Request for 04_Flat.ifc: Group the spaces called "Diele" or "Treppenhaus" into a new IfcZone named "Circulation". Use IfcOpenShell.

First a look at what the model holds.

```python
import ifcopenshell

model = ifcopenshell.open("04_Flat.ifc")
print(model.schema)
seen = {}
for space in model.by_type("IfcSpace"):
    seen[space.LongName] = seen.get(space.LongName, 0) + 1
for name, count in sorted(seen.items(), key=str):
    print(count, "x", name)
print("zones:", [z.Name for z in model.by_type("IfcZone")][:20])
```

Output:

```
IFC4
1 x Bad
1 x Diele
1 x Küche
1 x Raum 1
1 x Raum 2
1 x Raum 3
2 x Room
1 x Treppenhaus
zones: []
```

```python
import ifcopenshell
import ifcopenshell.api.group
import ifcopenshell.api.root

model = ifcopenshell.open("04_Flat.ifc")

names = {"Diele", "Treppenhaus"}
spaces = [s for s in model.by_type("IfcSpace") if s.LongName in names]

zone = ifcopenshell.api.root.create_entity(model, ifc_class="IfcZone", name="Circulation")
ifcopenshell.api.group.assign_group(model, products=spaces, group=zone)
print(len(spaces), "spaces in", zone.Name)

model.write("04_Flat_updated.ifc")
```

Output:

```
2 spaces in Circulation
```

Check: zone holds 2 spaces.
